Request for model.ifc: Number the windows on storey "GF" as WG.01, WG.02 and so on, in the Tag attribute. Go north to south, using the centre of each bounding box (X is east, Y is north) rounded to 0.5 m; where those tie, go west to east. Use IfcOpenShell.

First a look at what the model holds.

```python
import ifcopenshell
import ifcopenshell.util.element
import ifcopenshell.util.placement

model = ifcopenshell.open("model.ifc")
print(model.schema)
storey = next(s for s in model.by_type("IfcBuildingStorey") if s.Name == "GF")
windows = [e for e in ifcopenshell.util.element.get_decomposition(storey) if e.is_a("IfcWindow")]
for e in sorted(windows, key=lambda e: e.id()):
    origin = ifcopenshell.util.placement.get_local_placement(e.ObjectPlacement)[:3, 3]
    print(e.id(), e.Tag, e.Name, origin.round(2) + 0.0, sep=" | ")
```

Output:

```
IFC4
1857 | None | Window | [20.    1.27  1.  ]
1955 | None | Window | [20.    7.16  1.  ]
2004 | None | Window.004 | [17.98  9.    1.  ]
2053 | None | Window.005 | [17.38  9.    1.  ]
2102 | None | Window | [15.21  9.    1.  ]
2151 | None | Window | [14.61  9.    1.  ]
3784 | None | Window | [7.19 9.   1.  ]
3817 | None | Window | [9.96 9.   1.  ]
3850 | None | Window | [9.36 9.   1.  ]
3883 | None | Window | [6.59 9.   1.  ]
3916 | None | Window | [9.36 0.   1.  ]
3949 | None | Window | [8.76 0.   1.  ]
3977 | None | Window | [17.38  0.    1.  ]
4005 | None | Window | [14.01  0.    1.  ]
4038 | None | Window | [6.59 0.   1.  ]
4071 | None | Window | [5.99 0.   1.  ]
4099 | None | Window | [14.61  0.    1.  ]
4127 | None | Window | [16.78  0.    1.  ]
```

```python
import ifcopenshell
import ifcopenshell.geom
import ifcopenshell.util.element
import ifcopenshell.util.shape

model = ifcopenshell.open("model.ifc")
settings = ifcopenshell.geom.settings()
settings.set("use-world-coords", True)


def centre(element):
    shape = ifcopenshell.geom.create_shape(settings, element)
    return ifcopenshell.util.shape.get_bbox_centroid(shape.geometry)


storey = next(s for s in model.by_type("IfcBuildingStorey") if s.Name == "GF")
windows = [e for e in ifcopenshell.util.element.get_decomposition(storey) if e.is_a("IfcWindow")]

# Insertion points can sit at a corner or the storey origin, so sort by the geometry (in metres).
centres = {e: centre(e) for e in windows}
windows.sort(key=lambda e: (-round(centres[e][1] / 0.5), centres[e][0]))

for i, e in enumerate(windows, start=1):
    number = f"WG.{i:02d}"
    e.Tag = number
    print(e.id(), number)

model.write("model_updated.ifc")
```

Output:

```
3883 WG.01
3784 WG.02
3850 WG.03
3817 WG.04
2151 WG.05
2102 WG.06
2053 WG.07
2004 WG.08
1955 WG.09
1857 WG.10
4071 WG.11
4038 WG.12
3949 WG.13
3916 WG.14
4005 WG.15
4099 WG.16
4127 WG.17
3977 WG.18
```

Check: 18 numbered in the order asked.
